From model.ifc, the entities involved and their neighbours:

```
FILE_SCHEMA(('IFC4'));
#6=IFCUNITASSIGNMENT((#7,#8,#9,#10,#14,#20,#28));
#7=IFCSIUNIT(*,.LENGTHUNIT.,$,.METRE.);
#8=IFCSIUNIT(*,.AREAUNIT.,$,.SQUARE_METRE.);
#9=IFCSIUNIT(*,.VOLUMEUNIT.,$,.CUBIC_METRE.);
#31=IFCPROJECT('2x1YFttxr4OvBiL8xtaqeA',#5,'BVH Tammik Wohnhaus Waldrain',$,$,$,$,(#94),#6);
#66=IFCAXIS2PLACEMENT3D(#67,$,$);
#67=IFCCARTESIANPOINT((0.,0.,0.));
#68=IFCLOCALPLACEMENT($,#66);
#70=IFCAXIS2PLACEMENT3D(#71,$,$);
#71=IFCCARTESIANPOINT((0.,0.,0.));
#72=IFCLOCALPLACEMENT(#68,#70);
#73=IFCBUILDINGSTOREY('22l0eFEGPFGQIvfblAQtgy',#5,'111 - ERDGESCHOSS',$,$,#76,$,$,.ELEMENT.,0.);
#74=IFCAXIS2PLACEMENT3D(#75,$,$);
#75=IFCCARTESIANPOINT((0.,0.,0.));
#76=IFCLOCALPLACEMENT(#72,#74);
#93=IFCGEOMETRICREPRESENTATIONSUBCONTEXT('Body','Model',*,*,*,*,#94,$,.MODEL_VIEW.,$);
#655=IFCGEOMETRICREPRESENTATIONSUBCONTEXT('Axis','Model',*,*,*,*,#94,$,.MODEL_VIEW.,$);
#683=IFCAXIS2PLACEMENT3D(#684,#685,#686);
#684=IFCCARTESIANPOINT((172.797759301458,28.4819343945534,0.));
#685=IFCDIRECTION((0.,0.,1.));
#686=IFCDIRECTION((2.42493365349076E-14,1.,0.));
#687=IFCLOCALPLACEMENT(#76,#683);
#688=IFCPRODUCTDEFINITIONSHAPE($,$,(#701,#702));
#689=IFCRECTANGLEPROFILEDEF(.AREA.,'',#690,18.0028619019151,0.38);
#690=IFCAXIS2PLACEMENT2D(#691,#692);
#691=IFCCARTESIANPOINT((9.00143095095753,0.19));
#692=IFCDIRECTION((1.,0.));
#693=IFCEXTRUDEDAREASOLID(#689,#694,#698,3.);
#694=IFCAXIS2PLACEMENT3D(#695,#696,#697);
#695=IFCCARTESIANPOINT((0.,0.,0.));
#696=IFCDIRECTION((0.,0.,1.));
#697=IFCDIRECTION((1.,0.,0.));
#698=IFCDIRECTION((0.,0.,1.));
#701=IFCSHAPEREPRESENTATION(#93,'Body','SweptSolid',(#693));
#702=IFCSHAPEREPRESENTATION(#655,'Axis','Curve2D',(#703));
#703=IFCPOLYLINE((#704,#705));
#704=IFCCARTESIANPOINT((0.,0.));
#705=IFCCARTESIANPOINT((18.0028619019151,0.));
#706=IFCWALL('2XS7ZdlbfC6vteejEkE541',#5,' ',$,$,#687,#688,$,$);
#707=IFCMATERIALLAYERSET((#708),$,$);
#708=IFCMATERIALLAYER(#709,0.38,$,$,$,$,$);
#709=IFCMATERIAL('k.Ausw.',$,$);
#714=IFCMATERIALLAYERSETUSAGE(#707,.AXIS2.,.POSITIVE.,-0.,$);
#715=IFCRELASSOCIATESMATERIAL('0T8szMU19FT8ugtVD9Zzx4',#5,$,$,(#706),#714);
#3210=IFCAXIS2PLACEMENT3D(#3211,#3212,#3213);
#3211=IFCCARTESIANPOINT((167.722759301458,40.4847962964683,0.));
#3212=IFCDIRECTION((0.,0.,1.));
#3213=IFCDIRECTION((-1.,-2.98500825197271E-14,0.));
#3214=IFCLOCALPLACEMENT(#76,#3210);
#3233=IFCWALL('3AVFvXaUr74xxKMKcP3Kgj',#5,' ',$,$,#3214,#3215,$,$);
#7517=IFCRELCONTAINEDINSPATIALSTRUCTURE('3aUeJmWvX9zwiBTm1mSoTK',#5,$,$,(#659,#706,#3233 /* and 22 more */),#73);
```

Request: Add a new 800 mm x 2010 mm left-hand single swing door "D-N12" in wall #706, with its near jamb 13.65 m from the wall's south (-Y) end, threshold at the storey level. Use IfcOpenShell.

```python
import numpy as np
import ifcopenshell
import ifcopenshell.api.feature
import ifcopenshell.api.geometry
import ifcopenshell.api.root
import ifcopenshell.api.spatial
import ifcopenshell.geom
import ifcopenshell.util.element
import ifcopenshell.util.placement
import ifcopenshell.util.representation
import ifcopenshell.util.shape
import ifcopenshell.util.unit

model = ifcopenshell.open("model.ifc")
unit_scale = ifcopenshell.util.unit.calculate_unit_scale(model)
settings = ifcopenshell.geom.settings()


def volume(element):
    """Net volume in cubic metres, openings subtracted."""
    shape = ifcopenshell.geom.create_shape(settings, element)
    return ifcopenshell.util.shape.get_volume(shape.geometry)


wall = model.by_guid("2XS7ZdlbfC6vteejEkE541")
storey = ifcopenshell.util.element.get_container(wall, ifc_class="IfcBuildingStorey")
context = ifcopenshell.util.representation.get_context(model, "Model", "Body", "MODEL_VIEW")
before = volume(wall)

width, height, from_end, sill = 0.8, 2.01, 13.65, 0.0  # metres

# The wall runs along its own X axis, and the end named is its -X end.
wall_shape = ifcopenshell.geom.create_shape(settings, wall)
x, y, z = ifcopenshell.util.shape.get_vertices(wall_shape.geometry).T
start = x.min() + from_end
face, thickness = float(y.min()), float(y.max() - y.min())
wall_matrix = ifcopenshell.util.placement.get_local_placement(wall.ObjectPlacement)
level = ifcopenshell.util.placement.get_local_placement(storey.ObjectPlacement)[2, 3]


def in_wall(x, y):
    """Placement at x, y metres in the wall's axes, at sill height."""
    matrix = wall_matrix.copy()
    matrix[:, 3] = wall_matrix @ np.array([x / unit_scale, y / unit_scale, 0.0, 1.0])
    matrix[2, 3] = level + sill / unit_scale
    return matrix


# Opening: a box that overshoots both wall faces by 50 mm.
opening = ifcopenshell.api.root.create_entity(model, ifc_class="IfcOpeningElement", predefined_type="OPENING")
box = ifcopenshell.api.geometry.add_wall_representation(
    model, context=context, length=width, height=height, thickness=thickness + 0.1
)
ifcopenshell.api.geometry.assign_representation(model, product=opening, representation=box)
ifcopenshell.api.geometry.edit_object_placement(model, product=opening, matrix=in_wall(start, face - 0.05), is_si=False)
ifcopenshell.api.feature.add_feature(model, feature=opening, element=wall)

door = ifcopenshell.api.root.create_entity(model, ifc_class="IfcDoor", name="D-N12", predefined_type="DOOR")
door.OverallWidth, door.OverallHeight = width / unit_scale, height / unit_scale
door.OperationType = "SINGLE_SWING_LEFT"
body = ifcopenshell.api.geometry.add_door_representation(
    model,
    context=context,
    overall_width=door.OverallWidth,
    overall_height=door.OverallHeight,
    operation_type="SINGLE_SWING_LEFT",
    lining_properties={"LiningDepth": thickness / unit_scale, "ThresholdDepth": thickness / unit_scale},
)
ifcopenshell.api.geometry.assign_representation(model, product=door, representation=body)
ifcopenshell.api.spatial.assign_container(model, products=[door], relating_structure=storey)
ifcopenshell.api.feature.add_filling(model, opening=opening, element=door)

# The lining spans the wall, so the door starts at the wall face.
ifcopenshell.api.geometry.edit_object_placement(model, product=door, matrix=in_wall(start, face), is_si=False)

after = volume(wall)

print(f"wall volume {before:.3f} -> {after:.3f} m3")

model.write("model-out.ifc")
```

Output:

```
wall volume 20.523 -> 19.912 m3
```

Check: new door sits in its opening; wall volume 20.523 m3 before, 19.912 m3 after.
